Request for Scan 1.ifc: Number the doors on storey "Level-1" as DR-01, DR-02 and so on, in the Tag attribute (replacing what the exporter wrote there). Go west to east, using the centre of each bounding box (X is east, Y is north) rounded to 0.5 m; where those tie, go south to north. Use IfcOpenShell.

First a look at what the model holds.

```python
import ifcopenshell
import ifcopenshell.util.element
import ifcopenshell.util.placement

model = ifcopenshell.open("Scan 1.ifc")
print(model.schema)
storey = next(s for s in model.by_type("IfcBuildingStorey") if s.Name == "Level-1")
doors = [e for e in ifcopenshell.util.element.get_decomposition(storey) if e.is_a("IfcDoor")]
for e in sorted(doors, key=lambda e: e.id()):
    origin = ifcopenshell.util.placement.get_local_placement(e.ObjectPlacement)[:3, 3]
    print(e.id(), e.Tag, e.Name, origin.round(2) + 0.0, sep=" | ")
```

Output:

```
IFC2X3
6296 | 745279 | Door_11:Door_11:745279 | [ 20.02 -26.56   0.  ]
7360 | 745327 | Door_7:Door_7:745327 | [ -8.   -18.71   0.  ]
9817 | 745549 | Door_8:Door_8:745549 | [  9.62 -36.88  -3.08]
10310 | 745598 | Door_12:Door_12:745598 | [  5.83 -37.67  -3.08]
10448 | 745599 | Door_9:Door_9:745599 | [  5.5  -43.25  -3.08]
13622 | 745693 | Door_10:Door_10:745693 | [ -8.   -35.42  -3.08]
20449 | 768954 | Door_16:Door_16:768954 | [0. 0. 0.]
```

```python
import ifcopenshell
import ifcopenshell.geom
import ifcopenshell.util.element
import ifcopenshell.util.shape

model = ifcopenshell.open("Scan 1.ifc")
settings = ifcopenshell.geom.settings()
settings.set("use-world-coords", True)


def centre(element):
    shape = ifcopenshell.geom.create_shape(settings, element)
    return ifcopenshell.util.shape.get_bbox_centroid(shape.geometry)


storey = next(s for s in model.by_type("IfcBuildingStorey") if s.Name == "Level-1")
doors = [e for e in ifcopenshell.util.element.get_decomposition(storey) if e.is_a("IfcDoor")]

# Insertion points can sit at a corner or the storey origin, so sort by the geometry (in metres).
centres = {e: centre(e) for e in doors}
doors.sort(key=lambda e: (round(centres[e][0] / 0.5), centres[e][1]))

for i, e in enumerate(doors, start=1):
    number = f"DR-{i:02d}"
    e.Tag = number
    print(e.id(), number)

model.write("Scan 1_edited.ifc")
```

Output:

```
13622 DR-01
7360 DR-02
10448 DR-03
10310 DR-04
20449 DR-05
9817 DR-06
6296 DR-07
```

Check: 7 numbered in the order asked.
